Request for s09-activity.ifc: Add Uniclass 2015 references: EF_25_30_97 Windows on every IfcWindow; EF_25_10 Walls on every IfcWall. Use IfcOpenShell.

First a look at what the model holds.

```python
import ifcopenshell

model = ifcopenshell.open("s09-activity.ifc")
print(model.schema)
print("classifications:", [c.Name for c in model.by_type("IfcClassification")])
for ifc_class in ("IfcDoor", "IfcRoof", "IfcStair", "IfcWall", "IfcWindow"):
    print(ifc_class, len(model.by_type(ifc_class)))
```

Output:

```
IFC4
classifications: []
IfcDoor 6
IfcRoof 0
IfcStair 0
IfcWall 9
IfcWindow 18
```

```python
import ifcopenshell
import ifcopenshell.api.classification

model = ifcopenshell.open("s09-activity.ifc")

system = ifcopenshell.api.classification.add_classification(model, classification="Uniclass 2015")

codes = {
    "IfcWindow": ("EF_25_30_97", "Windows"),
    "IfcWall": ("EF_25_10", "Walls"),
}
for ifc_class, (code, name) in codes.items():
    products = model.by_type(ifc_class)
    ifcopenshell.api.classification.add_reference(
        model, products=products, classification=system, identification=code, name=name
    )
    print(code, len(products))

model.write("s09-activity_rev.ifc")
```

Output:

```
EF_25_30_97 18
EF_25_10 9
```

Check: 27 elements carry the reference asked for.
